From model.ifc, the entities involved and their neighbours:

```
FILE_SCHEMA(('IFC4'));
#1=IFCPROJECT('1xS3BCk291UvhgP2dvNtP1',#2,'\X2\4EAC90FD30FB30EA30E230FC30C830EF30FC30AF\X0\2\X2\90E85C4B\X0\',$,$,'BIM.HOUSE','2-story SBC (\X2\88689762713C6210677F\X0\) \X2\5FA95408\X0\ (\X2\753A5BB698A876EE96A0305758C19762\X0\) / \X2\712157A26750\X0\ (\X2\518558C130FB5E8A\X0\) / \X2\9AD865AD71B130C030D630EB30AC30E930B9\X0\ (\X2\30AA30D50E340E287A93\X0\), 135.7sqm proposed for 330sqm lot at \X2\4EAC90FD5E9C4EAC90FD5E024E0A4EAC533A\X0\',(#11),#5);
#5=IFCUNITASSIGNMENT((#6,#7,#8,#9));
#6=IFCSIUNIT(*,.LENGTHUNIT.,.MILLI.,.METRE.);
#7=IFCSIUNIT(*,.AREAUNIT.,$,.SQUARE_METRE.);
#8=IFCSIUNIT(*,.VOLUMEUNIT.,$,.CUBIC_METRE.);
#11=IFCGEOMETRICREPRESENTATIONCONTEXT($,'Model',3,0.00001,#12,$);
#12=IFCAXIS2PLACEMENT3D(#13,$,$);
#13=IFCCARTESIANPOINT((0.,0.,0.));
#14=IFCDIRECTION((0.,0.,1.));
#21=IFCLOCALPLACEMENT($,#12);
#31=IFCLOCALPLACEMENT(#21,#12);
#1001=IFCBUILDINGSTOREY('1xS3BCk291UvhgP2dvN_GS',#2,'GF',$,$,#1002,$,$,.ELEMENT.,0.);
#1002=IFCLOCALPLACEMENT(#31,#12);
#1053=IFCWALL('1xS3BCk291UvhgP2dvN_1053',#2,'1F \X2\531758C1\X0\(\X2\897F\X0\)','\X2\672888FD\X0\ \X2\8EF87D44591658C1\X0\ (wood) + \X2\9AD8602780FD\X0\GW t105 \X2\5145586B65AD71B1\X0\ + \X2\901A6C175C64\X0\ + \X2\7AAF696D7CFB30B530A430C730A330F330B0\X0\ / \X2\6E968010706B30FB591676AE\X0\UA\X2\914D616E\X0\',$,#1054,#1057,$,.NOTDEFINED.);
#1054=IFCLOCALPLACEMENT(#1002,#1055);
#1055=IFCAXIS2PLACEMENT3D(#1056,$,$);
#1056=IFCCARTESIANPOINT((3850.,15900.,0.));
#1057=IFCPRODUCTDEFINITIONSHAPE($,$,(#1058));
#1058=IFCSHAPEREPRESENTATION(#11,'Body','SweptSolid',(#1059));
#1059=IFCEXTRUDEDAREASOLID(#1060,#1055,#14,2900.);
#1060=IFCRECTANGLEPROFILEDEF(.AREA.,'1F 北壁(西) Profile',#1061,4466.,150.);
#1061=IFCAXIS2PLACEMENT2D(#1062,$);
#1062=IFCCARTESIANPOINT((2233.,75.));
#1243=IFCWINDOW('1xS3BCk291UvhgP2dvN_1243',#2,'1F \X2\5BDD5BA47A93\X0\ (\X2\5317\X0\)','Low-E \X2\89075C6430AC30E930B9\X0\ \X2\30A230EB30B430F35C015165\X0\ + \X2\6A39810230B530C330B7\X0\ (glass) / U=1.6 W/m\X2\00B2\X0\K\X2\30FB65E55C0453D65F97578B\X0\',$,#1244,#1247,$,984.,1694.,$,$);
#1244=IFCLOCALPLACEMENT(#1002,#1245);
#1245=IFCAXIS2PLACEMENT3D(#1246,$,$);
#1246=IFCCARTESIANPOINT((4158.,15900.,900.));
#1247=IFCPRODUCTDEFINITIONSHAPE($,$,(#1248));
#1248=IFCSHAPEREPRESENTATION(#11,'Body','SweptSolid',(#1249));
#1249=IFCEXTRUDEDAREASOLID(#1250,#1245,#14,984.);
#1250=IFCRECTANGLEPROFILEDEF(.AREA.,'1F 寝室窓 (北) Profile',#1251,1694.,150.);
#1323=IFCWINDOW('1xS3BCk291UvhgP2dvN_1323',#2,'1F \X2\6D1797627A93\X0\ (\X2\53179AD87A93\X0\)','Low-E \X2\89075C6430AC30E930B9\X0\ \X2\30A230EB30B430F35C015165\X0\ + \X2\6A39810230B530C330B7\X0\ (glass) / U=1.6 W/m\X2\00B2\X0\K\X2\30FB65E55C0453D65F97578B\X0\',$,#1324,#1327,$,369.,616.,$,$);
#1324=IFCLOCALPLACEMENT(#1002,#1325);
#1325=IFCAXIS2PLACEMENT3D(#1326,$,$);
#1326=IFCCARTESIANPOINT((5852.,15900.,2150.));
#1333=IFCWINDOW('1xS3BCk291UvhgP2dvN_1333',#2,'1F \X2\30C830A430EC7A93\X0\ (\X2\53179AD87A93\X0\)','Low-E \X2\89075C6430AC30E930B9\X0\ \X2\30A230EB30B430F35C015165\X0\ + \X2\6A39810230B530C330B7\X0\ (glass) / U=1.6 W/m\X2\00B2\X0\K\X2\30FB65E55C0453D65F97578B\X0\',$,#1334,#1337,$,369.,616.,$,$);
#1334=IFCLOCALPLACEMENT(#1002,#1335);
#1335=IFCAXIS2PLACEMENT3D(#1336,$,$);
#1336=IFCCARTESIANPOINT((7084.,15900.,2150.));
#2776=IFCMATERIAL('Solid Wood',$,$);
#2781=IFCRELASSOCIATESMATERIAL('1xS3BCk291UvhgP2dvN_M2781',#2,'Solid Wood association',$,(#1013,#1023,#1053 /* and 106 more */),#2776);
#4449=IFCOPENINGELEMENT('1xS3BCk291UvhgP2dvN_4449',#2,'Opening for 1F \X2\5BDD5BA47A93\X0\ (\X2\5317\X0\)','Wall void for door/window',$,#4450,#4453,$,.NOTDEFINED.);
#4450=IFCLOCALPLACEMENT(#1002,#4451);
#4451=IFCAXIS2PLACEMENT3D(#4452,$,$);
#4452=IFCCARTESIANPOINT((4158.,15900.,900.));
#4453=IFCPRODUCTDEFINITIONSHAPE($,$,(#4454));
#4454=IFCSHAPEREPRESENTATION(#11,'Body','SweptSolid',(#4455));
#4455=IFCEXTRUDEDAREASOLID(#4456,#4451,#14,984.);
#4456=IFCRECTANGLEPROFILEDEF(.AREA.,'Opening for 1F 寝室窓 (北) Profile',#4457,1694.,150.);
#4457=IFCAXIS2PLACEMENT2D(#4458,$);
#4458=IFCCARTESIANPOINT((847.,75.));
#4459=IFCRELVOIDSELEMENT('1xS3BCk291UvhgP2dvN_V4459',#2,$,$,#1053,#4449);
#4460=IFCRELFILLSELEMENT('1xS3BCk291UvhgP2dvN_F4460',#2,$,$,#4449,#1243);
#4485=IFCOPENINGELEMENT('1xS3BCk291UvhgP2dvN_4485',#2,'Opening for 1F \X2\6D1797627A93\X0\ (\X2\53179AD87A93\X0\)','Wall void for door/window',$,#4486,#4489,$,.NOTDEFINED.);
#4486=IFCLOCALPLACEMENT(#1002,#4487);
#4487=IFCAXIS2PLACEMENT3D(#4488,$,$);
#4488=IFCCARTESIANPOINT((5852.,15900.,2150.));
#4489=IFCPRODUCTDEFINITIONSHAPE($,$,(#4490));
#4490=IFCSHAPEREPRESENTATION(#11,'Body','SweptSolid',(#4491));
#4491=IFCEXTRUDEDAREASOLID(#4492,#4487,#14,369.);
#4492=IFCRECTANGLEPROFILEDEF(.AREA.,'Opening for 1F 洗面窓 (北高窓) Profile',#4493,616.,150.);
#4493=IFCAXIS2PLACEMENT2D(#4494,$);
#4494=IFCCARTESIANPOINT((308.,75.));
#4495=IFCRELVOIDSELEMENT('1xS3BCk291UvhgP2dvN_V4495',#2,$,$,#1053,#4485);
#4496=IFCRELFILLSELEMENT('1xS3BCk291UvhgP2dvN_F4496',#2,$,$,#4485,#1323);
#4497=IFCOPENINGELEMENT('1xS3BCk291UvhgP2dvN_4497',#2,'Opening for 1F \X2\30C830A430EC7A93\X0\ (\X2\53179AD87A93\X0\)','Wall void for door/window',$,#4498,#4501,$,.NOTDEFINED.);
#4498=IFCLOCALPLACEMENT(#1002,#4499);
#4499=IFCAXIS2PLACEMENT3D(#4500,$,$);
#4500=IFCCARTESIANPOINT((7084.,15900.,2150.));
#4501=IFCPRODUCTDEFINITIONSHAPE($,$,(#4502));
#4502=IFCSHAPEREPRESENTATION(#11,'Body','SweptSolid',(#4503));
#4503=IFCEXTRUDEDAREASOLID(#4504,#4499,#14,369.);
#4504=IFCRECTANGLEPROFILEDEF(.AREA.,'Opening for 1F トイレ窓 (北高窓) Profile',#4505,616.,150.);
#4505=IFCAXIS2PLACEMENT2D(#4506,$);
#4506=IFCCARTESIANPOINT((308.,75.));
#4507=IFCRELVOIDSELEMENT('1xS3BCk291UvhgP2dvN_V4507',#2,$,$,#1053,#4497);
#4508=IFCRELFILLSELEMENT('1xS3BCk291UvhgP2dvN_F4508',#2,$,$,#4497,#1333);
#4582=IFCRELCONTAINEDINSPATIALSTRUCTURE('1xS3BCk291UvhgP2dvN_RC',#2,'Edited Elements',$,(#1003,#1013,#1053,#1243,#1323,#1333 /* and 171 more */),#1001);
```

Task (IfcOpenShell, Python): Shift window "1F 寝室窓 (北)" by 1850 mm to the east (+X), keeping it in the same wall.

```python
import ifcopenshell
import ifcopenshell.api.geometry
import ifcopenshell.util.placement
import ifcopenshell.util.unit

model = ifcopenshell.open("model.ifc")
unit_scale = ifcopenshell.util.unit.calculate_unit_scale(model)

window = model.by_guid("1xS3BCk291UvhgP2dvN_1243")
opening = window.FillsVoids[0].RelatingOpeningElement
wall = opening.VoidsElements[0].RelatingBuildingElement

wall_matrix = ifcopenshell.util.placement.get_local_placement(wall.ObjectPlacement)
shift = wall_matrix[:3, 0] * 1.85 / unit_scale
before = ifcopenshell.util.placement.get_local_placement(window.ObjectPlacement)[:3, 3].copy()

# The window is not placed relative to its opening, so move both.
for product in (opening, window):
    matrix = ifcopenshell.util.placement.get_local_placement(product.ObjectPlacement)
    matrix[:3, 3] += shift
    ifcopenshell.api.geometry.edit_object_placement(model, product=product, matrix=matrix, is_si=False)

after = ifcopenshell.util.placement.get_local_placement(window.ObjectPlacement)[:3, 3]
print("window moved by", (after - before).round(3) + 0.0)

model.write("model_v2.ifc")
```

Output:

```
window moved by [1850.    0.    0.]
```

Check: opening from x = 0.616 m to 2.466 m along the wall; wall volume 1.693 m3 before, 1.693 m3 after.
